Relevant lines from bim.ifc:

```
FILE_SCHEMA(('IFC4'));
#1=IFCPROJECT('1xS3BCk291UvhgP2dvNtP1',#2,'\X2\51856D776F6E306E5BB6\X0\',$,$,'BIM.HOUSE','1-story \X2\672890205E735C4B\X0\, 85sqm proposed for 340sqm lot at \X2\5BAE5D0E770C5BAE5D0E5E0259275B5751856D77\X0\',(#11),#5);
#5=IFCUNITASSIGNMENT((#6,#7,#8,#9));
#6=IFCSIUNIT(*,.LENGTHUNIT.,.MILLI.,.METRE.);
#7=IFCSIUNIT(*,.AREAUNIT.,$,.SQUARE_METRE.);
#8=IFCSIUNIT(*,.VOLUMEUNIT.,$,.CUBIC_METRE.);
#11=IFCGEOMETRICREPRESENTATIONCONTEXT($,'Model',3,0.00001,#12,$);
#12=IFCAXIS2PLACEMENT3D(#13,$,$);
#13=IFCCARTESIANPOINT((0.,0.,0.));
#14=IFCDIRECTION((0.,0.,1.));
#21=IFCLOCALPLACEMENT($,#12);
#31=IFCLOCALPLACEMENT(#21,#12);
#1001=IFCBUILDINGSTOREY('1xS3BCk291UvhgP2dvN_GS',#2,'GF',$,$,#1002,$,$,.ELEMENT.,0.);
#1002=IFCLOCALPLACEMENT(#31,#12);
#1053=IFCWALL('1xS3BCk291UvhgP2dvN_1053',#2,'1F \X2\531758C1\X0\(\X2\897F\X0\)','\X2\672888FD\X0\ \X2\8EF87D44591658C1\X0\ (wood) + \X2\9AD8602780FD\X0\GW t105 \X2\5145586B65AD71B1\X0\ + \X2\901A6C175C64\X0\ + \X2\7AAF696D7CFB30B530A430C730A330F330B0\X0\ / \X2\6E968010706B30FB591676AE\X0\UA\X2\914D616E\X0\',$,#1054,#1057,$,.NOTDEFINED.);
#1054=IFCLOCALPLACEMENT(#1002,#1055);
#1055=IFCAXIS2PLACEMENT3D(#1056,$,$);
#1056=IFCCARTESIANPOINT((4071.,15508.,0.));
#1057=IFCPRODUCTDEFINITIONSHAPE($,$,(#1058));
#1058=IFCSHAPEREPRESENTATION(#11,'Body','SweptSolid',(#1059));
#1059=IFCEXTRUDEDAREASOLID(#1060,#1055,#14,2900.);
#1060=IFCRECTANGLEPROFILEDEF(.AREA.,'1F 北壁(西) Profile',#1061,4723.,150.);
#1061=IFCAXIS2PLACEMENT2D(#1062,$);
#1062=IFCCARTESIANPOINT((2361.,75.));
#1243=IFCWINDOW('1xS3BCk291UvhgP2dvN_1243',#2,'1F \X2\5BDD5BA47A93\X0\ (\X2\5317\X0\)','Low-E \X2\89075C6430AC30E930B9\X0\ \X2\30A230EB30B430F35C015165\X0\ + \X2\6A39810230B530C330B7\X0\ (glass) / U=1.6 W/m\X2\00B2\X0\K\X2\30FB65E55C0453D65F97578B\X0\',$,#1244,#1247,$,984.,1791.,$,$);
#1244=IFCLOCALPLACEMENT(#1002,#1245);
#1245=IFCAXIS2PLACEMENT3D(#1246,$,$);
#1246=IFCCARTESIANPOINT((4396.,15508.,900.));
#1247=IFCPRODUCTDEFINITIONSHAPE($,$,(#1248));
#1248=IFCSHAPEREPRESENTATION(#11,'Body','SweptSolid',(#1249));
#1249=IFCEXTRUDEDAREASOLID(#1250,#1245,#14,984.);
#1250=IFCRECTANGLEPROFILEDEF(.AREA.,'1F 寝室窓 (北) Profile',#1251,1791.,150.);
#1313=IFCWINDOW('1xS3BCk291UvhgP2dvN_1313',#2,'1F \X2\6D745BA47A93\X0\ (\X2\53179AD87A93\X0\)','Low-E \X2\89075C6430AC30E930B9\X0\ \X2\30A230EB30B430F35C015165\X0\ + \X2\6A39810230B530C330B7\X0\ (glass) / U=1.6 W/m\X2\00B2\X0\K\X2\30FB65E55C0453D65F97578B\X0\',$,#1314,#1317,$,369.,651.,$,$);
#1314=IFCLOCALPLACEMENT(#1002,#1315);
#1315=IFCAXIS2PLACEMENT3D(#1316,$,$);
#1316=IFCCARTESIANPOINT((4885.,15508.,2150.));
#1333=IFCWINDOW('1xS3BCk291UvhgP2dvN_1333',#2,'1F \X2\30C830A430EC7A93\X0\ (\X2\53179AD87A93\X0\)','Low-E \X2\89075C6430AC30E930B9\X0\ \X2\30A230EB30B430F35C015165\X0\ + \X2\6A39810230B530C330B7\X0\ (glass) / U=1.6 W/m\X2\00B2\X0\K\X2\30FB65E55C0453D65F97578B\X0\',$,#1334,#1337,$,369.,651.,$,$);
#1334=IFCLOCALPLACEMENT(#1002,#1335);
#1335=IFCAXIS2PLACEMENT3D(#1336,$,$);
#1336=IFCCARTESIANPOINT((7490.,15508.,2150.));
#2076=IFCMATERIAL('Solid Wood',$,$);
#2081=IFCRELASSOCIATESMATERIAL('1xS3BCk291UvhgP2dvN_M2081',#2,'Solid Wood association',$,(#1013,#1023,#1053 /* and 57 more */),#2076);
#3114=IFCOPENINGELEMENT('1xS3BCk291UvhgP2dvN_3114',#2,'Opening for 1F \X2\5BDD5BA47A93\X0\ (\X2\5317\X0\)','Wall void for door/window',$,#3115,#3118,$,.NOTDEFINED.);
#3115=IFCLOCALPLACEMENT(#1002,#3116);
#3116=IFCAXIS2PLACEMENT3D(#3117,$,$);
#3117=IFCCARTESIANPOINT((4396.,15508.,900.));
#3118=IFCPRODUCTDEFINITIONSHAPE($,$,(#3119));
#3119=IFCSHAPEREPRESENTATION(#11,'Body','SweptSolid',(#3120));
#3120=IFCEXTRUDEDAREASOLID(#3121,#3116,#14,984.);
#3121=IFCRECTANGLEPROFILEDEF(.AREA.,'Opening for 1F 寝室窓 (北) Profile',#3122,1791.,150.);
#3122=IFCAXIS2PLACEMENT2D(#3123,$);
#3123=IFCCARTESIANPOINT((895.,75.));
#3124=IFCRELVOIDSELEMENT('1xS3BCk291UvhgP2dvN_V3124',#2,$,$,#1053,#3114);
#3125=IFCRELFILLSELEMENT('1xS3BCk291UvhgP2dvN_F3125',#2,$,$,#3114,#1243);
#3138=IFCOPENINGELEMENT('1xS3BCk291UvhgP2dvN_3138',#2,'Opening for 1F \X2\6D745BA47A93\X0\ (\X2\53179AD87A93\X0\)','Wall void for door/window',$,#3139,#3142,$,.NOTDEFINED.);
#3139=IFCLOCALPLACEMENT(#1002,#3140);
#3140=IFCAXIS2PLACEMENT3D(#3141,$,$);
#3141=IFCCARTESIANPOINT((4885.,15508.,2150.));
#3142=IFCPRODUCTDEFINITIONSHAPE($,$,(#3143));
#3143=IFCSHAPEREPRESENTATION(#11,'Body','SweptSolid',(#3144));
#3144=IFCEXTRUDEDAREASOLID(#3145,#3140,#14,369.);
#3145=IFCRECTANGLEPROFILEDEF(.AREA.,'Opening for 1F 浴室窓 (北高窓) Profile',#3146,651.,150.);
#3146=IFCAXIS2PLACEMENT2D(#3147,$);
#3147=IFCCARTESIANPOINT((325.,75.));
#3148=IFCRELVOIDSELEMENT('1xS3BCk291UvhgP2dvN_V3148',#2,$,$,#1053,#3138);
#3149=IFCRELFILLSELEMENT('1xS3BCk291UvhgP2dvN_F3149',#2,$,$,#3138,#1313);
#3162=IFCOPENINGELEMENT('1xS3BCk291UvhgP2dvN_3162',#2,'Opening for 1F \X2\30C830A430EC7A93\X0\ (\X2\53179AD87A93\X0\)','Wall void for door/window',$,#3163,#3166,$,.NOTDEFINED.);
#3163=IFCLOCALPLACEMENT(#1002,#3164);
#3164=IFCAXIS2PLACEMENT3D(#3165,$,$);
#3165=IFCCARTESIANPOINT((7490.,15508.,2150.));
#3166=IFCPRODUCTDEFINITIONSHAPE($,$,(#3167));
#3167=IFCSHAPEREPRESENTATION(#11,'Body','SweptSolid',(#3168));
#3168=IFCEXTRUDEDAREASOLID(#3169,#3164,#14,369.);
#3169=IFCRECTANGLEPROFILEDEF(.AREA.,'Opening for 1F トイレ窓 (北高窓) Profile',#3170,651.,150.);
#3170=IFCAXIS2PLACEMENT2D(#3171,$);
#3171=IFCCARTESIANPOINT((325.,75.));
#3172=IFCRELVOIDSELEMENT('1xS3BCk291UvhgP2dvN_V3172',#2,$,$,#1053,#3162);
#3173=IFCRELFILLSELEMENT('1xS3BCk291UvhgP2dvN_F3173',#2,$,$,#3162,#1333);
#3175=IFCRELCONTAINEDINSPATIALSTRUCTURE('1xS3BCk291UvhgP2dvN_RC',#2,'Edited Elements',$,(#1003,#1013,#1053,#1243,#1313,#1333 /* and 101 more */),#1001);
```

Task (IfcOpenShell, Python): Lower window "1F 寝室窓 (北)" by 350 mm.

```python
import numpy as np
import ifcopenshell
import ifcopenshell.api.geometry
import ifcopenshell.util.placement
import ifcopenshell.util.unit

model = ifcopenshell.open("bim.ifc")
unit_scale = ifcopenshell.util.unit.calculate_unit_scale(model)

window = model.by_guid("1xS3BCk291UvhgP2dvN_1243")
opening = window.FillsVoids[0].RelatingOpeningElement
dz = -0.35 / unit_scale

shift = np.array([0.0, 0.0, dz])
# The window is not placed relative to its opening, so move both.
for product in (opening, window):
    matrix = ifcopenshell.util.placement.get_local_placement(product.ObjectPlacement)
    matrix[:3, 3] += shift
    ifcopenshell.api.geometry.edit_object_placement(model, product=product, matrix=matrix, is_si=False)

print(f"moved by {dz * unit_scale:+.3f} m")

model.write("bim-out.ifc")
```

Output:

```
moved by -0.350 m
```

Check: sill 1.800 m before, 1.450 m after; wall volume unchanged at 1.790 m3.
